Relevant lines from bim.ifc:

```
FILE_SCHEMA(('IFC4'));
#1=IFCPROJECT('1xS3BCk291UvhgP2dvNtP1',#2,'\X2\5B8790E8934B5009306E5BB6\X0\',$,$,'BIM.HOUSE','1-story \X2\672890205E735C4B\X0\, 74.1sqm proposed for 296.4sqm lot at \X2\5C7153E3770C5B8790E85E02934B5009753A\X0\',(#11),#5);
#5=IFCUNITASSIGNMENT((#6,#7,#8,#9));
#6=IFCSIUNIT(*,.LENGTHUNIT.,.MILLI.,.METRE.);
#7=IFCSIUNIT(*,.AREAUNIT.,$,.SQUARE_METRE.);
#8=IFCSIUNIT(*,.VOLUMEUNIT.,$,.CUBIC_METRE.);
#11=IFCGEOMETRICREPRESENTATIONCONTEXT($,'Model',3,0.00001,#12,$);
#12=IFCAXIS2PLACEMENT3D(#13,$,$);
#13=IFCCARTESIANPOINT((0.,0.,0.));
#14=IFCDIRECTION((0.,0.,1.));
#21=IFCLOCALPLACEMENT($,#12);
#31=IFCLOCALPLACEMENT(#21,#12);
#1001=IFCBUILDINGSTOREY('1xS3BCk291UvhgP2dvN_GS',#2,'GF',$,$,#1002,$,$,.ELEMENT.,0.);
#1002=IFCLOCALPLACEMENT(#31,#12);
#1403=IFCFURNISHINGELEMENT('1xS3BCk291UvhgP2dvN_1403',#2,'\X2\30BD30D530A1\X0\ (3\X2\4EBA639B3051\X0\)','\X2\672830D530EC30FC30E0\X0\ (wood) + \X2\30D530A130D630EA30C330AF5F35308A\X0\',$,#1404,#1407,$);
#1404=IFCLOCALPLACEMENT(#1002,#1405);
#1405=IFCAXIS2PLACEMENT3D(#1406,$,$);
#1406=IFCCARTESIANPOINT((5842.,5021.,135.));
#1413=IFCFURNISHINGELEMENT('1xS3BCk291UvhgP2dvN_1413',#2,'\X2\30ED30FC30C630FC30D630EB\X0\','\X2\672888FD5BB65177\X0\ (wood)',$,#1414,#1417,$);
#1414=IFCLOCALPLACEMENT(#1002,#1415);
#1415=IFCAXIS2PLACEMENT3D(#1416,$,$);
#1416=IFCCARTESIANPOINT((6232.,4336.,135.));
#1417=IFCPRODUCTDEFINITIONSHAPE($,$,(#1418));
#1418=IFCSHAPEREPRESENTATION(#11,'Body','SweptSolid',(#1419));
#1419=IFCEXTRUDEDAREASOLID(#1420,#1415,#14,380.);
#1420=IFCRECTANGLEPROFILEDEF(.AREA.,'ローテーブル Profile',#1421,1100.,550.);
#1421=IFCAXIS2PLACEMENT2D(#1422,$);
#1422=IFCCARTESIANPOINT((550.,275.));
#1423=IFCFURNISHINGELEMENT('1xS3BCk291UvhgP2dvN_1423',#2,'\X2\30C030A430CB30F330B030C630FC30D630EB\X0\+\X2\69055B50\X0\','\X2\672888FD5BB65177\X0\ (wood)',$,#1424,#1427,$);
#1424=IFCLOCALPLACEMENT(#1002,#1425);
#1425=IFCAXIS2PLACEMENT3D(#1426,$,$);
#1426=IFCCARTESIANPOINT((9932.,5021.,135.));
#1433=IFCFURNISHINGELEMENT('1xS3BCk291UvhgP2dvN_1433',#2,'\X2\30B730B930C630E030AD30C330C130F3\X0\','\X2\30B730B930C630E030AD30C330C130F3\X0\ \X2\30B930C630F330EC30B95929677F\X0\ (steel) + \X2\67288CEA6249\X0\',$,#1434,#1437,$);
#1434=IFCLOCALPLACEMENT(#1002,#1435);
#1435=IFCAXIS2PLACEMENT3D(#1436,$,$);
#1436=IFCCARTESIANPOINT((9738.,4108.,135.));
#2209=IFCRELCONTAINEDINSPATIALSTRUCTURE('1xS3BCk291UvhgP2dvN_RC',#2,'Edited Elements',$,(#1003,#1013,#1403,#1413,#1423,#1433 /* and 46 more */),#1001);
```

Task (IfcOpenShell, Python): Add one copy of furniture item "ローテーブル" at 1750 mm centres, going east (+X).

```python
import numpy as np
import ifcopenshell
import ifcopenshell.api.geometry
import ifcopenshell.api.root
import ifcopenshell.util.element
import ifcopenshell.util.placement

model = ifcopenshell.open("bim.ifc")


def reuse_history(source, copy):
    """copy_class also copies each property set's owner history, people and application; keep the originals."""
    for rel in copy.IsDefinedBy:
        if rel.is_a("IfcRelDefinesByProperties") and (history := rel.RelatingPropertyDefinition.OwnerHistory):
            rel.RelatingPropertyDefinition.OwnerHistory = source.OwnerHistory
            ifcopenshell.util.element.remove_deep2(model, history)


source = model.by_guid("1xS3BCk291UvhgP2dvN_1413")
base = ifcopenshell.util.placement.get_local_placement(source.ObjectPlacement)
step = np.array([1.0, 0.0, 0.0]) * 1750.0

for i in range(1, 2):
    copy = ifcopenshell.api.root.copy_class(model, product=source)
    copy.Representation = ifcopenshell.util.element.copy_deep(
        model, source.Representation, exclude=["IfcGeometricRepresentationContext", "IfcRepresentationMap"]
    )
    reuse_history(source, copy)
    matrix = base.copy()
    matrix[:3, 3] += i * step
    print("added at", matrix[:3, 3].round(3) + 0.0)
    ifcopenshell.api.geometry.edit_object_placement(model, product=copy, matrix=matrix, is_si=False)

model.write("bim_edited.ifc")
```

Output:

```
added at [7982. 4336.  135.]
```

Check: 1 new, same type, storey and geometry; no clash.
